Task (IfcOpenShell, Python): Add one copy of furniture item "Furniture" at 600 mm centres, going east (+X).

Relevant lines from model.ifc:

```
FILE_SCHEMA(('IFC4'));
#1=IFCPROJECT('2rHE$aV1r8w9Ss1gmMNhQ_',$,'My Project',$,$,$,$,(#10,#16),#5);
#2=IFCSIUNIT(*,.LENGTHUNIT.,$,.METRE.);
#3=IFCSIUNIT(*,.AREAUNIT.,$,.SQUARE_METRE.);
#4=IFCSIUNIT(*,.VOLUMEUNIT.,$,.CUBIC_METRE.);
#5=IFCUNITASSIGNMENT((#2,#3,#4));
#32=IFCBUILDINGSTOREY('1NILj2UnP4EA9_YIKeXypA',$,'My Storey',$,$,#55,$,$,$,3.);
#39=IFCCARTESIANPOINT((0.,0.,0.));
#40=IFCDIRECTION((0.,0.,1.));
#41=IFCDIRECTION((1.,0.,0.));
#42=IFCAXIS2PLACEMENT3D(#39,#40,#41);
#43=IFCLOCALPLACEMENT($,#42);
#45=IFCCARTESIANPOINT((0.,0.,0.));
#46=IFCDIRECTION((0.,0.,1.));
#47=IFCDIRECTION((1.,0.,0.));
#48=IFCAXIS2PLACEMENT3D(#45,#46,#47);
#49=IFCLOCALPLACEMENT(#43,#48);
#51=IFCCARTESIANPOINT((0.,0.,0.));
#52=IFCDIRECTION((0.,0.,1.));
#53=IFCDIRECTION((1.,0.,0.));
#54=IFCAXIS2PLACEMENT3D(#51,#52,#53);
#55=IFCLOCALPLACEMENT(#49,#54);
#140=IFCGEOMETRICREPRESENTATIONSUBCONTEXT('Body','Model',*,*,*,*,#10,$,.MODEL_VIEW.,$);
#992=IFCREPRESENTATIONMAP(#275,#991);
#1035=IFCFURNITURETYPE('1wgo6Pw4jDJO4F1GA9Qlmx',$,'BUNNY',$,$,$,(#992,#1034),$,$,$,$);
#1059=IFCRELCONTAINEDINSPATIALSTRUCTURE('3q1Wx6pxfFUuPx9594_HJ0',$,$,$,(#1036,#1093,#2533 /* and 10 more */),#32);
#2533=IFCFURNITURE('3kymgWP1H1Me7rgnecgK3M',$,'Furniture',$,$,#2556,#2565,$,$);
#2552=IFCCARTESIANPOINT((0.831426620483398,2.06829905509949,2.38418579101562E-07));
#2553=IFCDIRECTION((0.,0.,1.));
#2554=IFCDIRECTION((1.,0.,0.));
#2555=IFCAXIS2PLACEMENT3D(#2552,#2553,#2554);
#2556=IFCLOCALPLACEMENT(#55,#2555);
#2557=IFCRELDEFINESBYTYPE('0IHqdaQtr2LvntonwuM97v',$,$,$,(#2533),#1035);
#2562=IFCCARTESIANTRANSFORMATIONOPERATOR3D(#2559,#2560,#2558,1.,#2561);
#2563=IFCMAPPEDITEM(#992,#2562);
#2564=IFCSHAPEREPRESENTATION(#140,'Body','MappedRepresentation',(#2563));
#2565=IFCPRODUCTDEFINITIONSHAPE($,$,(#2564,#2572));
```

```python
import numpy as np
import ifcopenshell
import ifcopenshell.api.geometry
import ifcopenshell.api.root
import ifcopenshell.util.element
import ifcopenshell.util.placement
import ifcopenshell.util.unit

model = ifcopenshell.open("model.ifc")
unit_scale = ifcopenshell.util.unit.calculate_unit_scale(model)

source = model.by_id(2533)
base = ifcopenshell.util.placement.get_local_placement(source.ObjectPlacement)
step = np.array([1.0, 0.0, 0.0]) * 0.6 / unit_scale

for i in range(1, 2):
    copy = ifcopenshell.api.root.copy_class(model, product=source)
    copy.Representation = ifcopenshell.util.element.copy_deep(
        model, source.Representation, exclude=["IfcGeometricRepresentationContext", "IfcRepresentationMap"]
    )
    matrix = base.copy()
    matrix[:3, 3] += i * step
    print("added at", matrix[:3, 3].round(3) + 0.0)
    ifcopenshell.api.geometry.edit_object_placement(model, product=copy, matrix=matrix, is_si=False)

model.write("model-out.ifc")
```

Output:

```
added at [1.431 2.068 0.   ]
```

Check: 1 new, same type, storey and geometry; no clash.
